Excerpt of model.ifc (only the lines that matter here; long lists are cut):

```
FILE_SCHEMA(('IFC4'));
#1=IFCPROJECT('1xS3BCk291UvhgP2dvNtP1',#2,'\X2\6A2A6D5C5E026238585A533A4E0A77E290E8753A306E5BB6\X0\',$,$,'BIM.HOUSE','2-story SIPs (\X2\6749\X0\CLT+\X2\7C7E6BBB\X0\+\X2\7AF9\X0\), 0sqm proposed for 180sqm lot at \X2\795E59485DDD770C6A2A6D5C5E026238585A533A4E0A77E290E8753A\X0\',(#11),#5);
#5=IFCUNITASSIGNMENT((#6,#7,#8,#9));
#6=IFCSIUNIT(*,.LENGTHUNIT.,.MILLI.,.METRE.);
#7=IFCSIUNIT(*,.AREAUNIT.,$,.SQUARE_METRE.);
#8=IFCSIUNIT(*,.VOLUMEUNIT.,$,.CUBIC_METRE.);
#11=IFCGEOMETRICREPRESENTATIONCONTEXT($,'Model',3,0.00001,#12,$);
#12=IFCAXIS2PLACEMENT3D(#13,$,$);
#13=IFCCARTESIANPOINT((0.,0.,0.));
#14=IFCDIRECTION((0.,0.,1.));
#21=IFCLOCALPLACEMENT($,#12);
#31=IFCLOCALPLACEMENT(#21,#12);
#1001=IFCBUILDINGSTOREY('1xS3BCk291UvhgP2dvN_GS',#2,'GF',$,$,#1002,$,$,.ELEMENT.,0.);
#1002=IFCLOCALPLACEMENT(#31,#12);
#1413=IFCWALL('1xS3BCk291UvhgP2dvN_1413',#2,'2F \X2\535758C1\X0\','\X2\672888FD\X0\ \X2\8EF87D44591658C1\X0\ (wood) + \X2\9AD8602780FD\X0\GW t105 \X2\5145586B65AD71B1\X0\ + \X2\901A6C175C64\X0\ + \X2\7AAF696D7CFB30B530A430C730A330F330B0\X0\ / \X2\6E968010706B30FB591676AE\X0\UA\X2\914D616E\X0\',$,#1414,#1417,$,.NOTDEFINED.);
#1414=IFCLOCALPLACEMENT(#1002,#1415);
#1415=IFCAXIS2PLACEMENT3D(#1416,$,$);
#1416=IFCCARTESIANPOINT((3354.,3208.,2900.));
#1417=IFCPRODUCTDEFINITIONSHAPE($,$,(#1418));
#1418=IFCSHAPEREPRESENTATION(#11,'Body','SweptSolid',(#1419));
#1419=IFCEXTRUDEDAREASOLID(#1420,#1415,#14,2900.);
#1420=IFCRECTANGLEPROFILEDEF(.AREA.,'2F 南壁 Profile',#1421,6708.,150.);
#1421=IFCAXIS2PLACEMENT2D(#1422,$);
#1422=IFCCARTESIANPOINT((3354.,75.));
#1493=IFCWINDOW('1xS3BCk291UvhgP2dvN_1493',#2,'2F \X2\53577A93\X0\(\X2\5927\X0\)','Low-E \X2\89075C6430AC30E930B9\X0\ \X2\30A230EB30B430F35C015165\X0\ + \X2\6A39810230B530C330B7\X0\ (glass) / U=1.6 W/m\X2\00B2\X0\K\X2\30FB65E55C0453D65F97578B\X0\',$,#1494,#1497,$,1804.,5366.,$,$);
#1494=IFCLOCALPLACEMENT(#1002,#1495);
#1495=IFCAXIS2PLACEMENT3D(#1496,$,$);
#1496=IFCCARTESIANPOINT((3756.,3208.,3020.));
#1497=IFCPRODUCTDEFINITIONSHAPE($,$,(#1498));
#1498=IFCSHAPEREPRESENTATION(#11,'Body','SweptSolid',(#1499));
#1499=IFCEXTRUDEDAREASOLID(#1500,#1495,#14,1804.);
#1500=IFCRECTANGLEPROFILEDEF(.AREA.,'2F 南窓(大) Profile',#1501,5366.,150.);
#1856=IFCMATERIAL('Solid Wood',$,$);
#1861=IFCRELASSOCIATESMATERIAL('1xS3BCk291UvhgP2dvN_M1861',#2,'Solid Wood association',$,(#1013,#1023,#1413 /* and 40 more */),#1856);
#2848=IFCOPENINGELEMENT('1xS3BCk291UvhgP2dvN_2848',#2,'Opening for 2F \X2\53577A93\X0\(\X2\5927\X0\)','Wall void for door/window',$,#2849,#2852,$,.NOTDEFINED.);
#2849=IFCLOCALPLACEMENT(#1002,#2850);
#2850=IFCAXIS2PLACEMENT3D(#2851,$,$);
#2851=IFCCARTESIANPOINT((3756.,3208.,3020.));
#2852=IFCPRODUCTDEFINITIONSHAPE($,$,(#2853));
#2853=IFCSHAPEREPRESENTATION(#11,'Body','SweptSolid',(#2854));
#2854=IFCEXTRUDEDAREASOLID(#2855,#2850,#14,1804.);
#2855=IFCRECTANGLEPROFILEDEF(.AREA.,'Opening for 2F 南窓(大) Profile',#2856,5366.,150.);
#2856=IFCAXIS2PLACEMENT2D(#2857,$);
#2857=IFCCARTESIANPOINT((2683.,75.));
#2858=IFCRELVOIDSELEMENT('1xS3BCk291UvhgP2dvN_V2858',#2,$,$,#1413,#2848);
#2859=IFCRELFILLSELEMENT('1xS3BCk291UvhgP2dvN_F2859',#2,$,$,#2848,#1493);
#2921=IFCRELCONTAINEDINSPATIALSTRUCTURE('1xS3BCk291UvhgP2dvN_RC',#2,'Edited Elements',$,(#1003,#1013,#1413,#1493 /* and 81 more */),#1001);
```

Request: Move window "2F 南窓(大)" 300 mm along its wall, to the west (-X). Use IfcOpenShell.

```python
import ifcopenshell
import ifcopenshell.api.geometry
import ifcopenshell.util.placement
import ifcopenshell.util.unit

model = ifcopenshell.open("model.ifc")
unit_scale = ifcopenshell.util.unit.calculate_unit_scale(model)

window = model.by_id(1493)
opening = window.FillsVoids[0].RelatingOpeningElement
wall = opening.VoidsElements[0].RelatingBuildingElement

wall_matrix = ifcopenshell.util.placement.get_local_placement(wall.ObjectPlacement)
shift = wall_matrix[:3, 0] * -0.3 / unit_scale
before = ifcopenshell.util.placement.get_local_placement(window.ObjectPlacement)[:3, 3].copy()

# The window is not placed relative to its opening, so move both.
for product in (opening, window):
    matrix = ifcopenshell.util.placement.get_local_placement(product.ObjectPlacement)
    matrix[:3, 3] += shift
    ifcopenshell.api.geometry.edit_object_placement(model, product=product, matrix=matrix, is_si=False)

after = ifcopenshell.util.placement.get_local_placement(window.ObjectPlacement)[:3, 3]
print("window moved by", (after - before).round(3) + 0.0)

model.write("model_updated.ifc")
```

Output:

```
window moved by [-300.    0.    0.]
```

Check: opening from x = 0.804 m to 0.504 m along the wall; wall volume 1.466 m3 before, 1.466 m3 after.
